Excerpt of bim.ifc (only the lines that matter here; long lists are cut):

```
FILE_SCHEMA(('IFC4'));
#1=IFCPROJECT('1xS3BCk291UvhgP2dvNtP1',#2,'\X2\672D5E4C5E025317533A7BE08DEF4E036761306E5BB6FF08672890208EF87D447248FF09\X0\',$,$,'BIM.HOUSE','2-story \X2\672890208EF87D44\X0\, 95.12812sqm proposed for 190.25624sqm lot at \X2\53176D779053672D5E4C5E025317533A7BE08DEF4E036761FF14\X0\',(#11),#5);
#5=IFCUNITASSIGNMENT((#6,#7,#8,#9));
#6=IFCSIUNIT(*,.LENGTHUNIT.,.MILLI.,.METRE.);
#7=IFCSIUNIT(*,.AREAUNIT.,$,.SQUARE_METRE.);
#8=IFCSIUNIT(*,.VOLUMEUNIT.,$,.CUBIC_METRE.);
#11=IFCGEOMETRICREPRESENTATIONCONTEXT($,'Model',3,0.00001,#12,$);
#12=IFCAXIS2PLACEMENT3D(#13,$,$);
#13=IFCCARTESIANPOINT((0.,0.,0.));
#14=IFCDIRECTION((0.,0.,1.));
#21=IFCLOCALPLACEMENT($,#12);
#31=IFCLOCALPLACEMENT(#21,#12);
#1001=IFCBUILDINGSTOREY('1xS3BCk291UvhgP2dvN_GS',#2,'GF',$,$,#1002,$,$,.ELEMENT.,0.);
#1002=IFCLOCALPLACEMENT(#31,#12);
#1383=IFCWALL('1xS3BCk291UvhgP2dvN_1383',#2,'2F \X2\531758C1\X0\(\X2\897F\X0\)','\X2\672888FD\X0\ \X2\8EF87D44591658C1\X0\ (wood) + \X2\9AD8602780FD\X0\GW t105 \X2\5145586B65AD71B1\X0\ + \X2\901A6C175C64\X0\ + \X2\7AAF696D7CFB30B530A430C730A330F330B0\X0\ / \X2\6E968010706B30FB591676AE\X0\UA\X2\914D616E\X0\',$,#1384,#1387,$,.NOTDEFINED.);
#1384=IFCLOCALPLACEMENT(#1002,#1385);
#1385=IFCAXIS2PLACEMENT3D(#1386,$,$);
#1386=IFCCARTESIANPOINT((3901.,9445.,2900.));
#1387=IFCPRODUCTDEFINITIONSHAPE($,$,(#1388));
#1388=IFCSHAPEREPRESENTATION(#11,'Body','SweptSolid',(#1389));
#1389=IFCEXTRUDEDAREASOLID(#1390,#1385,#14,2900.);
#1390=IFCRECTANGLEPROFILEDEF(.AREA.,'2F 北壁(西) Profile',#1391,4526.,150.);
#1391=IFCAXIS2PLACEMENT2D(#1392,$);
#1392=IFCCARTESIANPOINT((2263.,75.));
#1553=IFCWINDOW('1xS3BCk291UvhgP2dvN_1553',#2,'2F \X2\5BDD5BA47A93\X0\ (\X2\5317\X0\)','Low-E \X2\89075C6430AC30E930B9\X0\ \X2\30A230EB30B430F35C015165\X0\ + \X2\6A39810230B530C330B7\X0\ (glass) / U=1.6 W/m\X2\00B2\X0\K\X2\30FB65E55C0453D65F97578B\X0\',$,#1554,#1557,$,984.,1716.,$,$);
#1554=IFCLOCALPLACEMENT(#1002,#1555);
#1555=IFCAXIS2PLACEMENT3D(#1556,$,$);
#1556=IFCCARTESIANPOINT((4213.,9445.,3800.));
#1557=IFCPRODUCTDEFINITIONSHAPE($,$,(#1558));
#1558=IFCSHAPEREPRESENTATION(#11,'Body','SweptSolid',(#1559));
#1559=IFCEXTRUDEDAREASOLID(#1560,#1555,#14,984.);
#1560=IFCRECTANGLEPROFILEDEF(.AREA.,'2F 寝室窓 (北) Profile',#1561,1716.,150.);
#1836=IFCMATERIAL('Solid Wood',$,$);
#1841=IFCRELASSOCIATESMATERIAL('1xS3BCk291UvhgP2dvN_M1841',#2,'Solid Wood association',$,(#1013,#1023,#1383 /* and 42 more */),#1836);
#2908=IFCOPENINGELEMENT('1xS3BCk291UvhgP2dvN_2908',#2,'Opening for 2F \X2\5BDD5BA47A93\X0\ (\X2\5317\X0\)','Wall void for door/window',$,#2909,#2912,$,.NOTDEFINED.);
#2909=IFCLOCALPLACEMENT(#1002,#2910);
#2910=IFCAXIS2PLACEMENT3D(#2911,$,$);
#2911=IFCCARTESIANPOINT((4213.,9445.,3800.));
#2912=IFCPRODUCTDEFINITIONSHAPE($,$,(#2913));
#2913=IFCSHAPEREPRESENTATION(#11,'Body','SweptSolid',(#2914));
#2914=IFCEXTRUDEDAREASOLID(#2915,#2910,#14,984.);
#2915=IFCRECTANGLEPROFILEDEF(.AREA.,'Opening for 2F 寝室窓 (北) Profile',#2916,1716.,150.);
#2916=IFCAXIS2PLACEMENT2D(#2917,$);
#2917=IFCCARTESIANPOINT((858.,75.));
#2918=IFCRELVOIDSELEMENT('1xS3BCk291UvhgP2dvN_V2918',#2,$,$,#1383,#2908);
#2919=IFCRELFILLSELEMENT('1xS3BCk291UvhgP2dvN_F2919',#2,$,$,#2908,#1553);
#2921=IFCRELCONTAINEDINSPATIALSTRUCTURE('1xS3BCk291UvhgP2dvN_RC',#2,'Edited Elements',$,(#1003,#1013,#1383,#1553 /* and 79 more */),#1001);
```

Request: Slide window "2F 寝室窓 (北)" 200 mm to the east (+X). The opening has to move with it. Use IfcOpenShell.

```python
import ifcopenshell
import ifcopenshell.api.geometry
import ifcopenshell.util.placement

model = ifcopenshell.open("bim.ifc")

window = model.by_guid("1xS3BCk291UvhgP2dvN_1553")
opening = window.FillsVoids[0].RelatingOpeningElement
wall = opening.VoidsElements[0].RelatingBuildingElement

wall_matrix = ifcopenshell.util.placement.get_local_placement(wall.ObjectPlacement)
shift = wall_matrix[:3, 0] * 200.0
before = ifcopenshell.util.placement.get_local_placement(window.ObjectPlacement)[:3, 3].copy()

# The window is not placed relative to its opening, so move both.
for product in (opening, window):
    matrix = ifcopenshell.util.placement.get_local_placement(product.ObjectPlacement)
    matrix[:3, 3] += shift
    ifcopenshell.api.geometry.edit_object_placement(model, product=product, matrix=matrix, is_si=False)

after = ifcopenshell.util.placement.get_local_placement(window.ObjectPlacement)[:3, 3]
print("window moved by", (after - before).round(3) + 0.0)

model.write("bim_edited.ifc")
```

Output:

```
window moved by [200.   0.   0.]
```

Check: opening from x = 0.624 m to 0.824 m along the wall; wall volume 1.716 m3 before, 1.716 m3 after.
